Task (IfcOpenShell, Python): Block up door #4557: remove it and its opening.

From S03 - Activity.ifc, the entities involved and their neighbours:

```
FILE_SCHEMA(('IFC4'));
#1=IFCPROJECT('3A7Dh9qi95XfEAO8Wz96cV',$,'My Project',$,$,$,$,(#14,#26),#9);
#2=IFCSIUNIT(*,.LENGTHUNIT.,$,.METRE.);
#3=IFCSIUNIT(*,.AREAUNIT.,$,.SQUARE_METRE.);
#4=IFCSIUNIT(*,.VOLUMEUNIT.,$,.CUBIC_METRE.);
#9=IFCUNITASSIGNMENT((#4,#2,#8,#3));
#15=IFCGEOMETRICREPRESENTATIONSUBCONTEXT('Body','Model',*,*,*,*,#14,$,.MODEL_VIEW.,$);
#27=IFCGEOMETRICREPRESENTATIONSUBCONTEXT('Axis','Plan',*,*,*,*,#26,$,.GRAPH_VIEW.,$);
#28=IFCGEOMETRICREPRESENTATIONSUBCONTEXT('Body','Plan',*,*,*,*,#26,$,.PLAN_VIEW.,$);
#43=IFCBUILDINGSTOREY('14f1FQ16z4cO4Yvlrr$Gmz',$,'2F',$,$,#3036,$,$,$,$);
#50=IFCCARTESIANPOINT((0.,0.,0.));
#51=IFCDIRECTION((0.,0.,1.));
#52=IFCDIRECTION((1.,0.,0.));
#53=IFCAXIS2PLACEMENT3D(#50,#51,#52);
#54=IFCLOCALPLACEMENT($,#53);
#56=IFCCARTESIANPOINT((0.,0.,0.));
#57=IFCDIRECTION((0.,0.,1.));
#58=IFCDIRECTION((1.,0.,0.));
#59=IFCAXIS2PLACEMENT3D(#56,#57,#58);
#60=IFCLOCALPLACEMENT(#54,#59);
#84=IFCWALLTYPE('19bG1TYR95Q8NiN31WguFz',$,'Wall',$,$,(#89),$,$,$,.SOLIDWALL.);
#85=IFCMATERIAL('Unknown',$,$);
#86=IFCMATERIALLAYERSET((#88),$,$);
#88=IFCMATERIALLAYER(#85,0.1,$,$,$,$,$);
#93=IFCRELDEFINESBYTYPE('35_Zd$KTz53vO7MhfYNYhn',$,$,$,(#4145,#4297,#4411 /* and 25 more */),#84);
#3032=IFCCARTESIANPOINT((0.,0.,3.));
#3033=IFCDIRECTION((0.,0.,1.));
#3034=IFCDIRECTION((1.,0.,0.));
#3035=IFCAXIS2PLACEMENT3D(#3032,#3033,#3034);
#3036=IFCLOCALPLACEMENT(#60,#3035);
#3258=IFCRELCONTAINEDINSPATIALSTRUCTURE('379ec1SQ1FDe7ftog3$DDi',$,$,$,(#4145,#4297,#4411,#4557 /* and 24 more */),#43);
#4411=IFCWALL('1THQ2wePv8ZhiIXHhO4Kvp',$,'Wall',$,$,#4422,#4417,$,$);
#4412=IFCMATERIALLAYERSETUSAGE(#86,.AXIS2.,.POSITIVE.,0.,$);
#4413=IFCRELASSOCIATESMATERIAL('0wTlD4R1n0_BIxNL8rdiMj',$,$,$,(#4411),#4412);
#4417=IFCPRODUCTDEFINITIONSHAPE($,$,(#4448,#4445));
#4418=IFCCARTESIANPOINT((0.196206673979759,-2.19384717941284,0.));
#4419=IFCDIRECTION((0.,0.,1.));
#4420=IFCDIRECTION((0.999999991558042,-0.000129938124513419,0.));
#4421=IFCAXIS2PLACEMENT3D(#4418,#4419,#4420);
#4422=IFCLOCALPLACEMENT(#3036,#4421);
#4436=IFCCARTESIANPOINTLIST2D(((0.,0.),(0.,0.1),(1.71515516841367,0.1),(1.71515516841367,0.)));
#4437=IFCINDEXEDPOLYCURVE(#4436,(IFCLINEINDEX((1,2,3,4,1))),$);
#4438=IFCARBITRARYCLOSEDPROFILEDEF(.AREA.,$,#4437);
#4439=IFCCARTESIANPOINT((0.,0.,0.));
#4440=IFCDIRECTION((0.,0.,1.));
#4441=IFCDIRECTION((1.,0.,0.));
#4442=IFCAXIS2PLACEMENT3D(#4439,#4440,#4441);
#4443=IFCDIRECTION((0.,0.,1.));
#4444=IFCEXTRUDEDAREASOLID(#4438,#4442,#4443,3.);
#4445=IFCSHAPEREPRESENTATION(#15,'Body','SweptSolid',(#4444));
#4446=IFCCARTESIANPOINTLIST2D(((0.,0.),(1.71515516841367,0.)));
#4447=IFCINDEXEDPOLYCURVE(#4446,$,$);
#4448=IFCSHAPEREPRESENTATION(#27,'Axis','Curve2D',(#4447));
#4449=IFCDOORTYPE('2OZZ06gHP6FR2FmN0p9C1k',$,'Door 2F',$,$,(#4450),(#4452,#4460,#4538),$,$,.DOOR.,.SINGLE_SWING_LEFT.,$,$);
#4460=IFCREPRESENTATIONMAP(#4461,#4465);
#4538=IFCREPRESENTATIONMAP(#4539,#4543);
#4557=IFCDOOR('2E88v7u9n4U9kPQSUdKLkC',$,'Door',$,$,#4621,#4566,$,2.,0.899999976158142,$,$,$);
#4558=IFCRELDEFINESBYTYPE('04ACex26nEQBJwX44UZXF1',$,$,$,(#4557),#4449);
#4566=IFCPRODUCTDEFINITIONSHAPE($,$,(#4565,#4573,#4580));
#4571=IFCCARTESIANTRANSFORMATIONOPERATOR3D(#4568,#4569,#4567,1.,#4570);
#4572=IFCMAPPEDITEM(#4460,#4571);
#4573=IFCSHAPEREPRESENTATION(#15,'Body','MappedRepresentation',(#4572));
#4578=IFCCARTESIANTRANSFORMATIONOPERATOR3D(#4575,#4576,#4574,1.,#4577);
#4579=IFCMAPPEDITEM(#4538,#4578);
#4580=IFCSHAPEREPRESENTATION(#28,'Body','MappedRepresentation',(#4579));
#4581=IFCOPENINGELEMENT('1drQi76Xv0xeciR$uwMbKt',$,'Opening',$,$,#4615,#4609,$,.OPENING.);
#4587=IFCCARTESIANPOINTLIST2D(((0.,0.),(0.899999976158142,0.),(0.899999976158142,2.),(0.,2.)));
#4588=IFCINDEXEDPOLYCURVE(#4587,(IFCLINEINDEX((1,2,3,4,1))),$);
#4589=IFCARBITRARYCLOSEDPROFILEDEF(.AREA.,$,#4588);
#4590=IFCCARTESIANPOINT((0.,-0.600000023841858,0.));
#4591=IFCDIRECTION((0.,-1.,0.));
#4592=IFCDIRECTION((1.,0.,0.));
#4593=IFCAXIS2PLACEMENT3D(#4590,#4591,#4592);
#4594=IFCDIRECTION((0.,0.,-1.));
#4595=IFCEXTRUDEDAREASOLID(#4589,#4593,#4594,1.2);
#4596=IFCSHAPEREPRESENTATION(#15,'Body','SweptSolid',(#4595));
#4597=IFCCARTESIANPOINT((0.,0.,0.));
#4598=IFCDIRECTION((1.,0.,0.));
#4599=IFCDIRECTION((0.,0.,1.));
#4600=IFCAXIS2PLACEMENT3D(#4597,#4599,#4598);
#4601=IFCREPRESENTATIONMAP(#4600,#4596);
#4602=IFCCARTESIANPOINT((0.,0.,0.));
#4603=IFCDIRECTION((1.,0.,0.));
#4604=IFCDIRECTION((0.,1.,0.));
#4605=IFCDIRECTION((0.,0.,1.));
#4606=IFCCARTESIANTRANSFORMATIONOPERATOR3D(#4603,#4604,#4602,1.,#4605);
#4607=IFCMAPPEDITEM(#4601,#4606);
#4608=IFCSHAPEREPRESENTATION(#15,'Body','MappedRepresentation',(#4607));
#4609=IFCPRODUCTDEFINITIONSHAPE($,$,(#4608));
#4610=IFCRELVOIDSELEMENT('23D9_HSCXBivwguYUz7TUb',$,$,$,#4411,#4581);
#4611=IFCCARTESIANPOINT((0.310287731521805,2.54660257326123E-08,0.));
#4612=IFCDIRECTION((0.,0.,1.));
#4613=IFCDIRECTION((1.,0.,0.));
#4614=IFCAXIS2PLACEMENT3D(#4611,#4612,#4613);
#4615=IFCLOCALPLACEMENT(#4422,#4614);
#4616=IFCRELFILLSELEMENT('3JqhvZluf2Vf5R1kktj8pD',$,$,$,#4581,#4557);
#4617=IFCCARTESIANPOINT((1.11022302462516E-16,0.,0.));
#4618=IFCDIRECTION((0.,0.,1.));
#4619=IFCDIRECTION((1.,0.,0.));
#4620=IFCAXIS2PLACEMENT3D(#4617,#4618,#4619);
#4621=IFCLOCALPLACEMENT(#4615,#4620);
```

```python
import ifcopenshell
import ifcopenshell.api.feature
import ifcopenshell.api.root
import ifcopenshell.geom
import ifcopenshell.util.shape

model = ifcopenshell.open("S03 - Activity.ifc")
settings = ifcopenshell.geom.settings()


def volume(element):
    """Net volume in cubic metres, openings subtracted."""
    shape = ifcopenshell.geom.create_shape(settings, element)
    return ifcopenshell.util.shape.get_volume(shape.geometry)


door = model.by_id(4557)
opening = door.FillsVoids[0].RelatingOpeningElement
wall = opening.VoidsElements[0].RelatingBuildingElement
before = volume(wall)

ifcopenshell.api.root.remove_product(model, product=door)
ifcopenshell.api.feature.remove_feature(model, feature=opening)

after = volume(wall)

print(f"wall volume {before:.3f} -> {after:.3f} m3")

model.write("S03 - Activity_v2.ifc")
```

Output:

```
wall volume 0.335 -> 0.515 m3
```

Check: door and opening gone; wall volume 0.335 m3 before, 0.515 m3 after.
